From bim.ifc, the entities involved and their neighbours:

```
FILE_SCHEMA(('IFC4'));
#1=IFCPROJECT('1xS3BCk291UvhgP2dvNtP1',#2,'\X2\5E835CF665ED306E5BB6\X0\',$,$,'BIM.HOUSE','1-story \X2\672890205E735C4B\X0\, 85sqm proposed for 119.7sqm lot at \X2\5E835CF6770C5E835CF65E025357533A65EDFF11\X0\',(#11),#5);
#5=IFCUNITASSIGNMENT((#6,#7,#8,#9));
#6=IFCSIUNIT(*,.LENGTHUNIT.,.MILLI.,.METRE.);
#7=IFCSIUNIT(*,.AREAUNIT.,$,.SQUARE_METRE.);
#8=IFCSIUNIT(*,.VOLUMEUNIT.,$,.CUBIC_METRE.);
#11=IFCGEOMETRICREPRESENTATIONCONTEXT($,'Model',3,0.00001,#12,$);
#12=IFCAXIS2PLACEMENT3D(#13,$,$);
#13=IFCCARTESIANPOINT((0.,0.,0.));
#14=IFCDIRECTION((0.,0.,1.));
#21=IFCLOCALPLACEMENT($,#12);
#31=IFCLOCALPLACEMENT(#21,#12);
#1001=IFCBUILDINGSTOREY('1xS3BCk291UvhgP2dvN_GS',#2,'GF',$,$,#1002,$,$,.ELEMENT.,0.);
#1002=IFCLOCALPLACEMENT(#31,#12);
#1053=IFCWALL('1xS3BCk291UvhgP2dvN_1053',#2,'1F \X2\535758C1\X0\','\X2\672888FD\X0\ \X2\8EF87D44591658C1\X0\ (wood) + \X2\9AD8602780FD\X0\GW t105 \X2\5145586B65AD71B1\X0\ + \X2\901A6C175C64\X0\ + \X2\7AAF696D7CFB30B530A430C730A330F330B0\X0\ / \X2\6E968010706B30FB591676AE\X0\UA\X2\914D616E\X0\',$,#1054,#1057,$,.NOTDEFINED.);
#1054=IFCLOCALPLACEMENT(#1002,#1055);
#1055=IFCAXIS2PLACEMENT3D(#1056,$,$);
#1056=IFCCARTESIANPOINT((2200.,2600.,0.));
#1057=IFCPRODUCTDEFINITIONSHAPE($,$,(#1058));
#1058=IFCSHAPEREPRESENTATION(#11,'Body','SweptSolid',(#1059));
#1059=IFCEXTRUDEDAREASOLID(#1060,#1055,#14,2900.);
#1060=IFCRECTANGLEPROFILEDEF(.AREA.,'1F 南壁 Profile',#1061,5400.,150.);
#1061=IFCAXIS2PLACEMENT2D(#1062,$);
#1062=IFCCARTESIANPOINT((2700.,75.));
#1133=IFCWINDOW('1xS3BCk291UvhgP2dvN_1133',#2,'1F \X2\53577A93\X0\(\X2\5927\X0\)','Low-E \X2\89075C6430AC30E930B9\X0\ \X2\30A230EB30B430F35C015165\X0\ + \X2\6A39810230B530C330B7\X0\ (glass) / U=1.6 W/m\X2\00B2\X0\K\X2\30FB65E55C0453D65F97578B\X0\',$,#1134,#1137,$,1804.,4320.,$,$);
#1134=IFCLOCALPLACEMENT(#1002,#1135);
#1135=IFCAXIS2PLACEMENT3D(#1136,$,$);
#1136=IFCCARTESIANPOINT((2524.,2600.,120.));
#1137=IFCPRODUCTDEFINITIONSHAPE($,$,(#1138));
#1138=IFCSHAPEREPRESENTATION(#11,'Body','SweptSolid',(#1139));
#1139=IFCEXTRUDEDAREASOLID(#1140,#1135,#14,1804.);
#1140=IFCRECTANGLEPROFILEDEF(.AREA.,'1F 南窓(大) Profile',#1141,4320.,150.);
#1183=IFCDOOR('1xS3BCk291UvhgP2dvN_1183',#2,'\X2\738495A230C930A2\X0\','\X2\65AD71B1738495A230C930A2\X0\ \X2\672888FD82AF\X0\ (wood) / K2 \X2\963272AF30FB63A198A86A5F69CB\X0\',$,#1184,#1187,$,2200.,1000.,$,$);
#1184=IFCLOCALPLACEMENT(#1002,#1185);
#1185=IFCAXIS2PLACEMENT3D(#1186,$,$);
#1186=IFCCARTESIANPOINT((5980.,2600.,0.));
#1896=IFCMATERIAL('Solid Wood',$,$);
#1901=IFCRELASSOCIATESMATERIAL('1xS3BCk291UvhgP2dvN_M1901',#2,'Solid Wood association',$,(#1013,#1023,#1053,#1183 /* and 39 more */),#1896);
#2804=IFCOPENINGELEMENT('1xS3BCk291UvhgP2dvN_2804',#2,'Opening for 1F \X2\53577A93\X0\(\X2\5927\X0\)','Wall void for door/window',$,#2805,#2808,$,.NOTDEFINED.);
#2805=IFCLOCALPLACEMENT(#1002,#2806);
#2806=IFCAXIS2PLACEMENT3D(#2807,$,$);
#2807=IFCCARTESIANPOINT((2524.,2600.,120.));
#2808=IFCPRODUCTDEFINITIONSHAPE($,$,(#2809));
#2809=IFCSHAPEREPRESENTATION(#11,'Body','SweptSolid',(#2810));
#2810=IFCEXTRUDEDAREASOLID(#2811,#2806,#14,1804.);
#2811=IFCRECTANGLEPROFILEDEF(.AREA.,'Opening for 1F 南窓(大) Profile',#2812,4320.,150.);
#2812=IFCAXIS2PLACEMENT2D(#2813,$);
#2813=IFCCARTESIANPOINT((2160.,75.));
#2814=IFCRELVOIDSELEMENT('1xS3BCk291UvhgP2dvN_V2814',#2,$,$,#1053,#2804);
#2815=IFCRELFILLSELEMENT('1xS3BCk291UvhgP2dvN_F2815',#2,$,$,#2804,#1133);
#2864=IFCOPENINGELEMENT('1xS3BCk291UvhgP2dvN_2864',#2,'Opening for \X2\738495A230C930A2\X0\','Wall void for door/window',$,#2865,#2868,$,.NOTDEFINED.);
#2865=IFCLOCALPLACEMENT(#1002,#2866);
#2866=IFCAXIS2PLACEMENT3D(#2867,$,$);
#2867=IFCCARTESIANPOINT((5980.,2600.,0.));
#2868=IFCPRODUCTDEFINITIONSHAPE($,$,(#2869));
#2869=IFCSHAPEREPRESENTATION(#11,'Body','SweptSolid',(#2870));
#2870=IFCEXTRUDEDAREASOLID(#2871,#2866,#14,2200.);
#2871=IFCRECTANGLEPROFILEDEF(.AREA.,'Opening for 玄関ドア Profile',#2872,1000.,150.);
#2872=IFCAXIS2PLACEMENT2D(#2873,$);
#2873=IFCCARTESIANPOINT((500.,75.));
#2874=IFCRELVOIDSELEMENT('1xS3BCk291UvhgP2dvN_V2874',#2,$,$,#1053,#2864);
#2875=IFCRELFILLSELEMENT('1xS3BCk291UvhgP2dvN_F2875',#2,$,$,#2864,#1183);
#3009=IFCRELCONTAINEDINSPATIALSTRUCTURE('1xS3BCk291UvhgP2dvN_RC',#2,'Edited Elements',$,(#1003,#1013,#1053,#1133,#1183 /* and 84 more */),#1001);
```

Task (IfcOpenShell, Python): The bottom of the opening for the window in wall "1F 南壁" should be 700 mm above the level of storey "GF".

```python
import numpy as np
import ifcopenshell
import ifcopenshell.api.geometry
import ifcopenshell.geom
import ifcopenshell.util.element
import ifcopenshell.util.placement
import ifcopenshell.util.shape
import ifcopenshell.util.unit

model = ifcopenshell.open("bim.ifc")
unit_scale = ifcopenshell.util.unit.calculate_unit_scale(model)

window = model.by_id(1133)
opening = window.FillsVoids[0].RelatingOpeningElement
storey = ifcopenshell.util.element.get_container(window, ifc_class="IfcBuildingStorey")
level = ifcopenshell.util.placement.get_local_placement(storey.ObjectPlacement)[2, 3]

# The opening's origin need not be at the sill, so measure its lowest point.
shape = ifcopenshell.geom.create_shape(ifcopenshell.geom.settings(), opening)
bottom = ifcopenshell.util.shape.get_shape_bottom_elevation(shape, shape.geometry) / unit_scale
dz = level + 700.0 - bottom

shift = np.array([0.0, 0.0, dz])
# The window is not placed relative to its opening, so move both.
for product in (opening, window):
    matrix = ifcopenshell.util.placement.get_local_placement(product.ObjectPlacement)
    matrix[:3, 3] += shift
    ifcopenshell.api.geometry.edit_object_placement(model, product=product, matrix=matrix, is_si=False)

print(f"moved by {dz * unit_scale:+.3f} m")

model.write("bim_v2.ifc")
```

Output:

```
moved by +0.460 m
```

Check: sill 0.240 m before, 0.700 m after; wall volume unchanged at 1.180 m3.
